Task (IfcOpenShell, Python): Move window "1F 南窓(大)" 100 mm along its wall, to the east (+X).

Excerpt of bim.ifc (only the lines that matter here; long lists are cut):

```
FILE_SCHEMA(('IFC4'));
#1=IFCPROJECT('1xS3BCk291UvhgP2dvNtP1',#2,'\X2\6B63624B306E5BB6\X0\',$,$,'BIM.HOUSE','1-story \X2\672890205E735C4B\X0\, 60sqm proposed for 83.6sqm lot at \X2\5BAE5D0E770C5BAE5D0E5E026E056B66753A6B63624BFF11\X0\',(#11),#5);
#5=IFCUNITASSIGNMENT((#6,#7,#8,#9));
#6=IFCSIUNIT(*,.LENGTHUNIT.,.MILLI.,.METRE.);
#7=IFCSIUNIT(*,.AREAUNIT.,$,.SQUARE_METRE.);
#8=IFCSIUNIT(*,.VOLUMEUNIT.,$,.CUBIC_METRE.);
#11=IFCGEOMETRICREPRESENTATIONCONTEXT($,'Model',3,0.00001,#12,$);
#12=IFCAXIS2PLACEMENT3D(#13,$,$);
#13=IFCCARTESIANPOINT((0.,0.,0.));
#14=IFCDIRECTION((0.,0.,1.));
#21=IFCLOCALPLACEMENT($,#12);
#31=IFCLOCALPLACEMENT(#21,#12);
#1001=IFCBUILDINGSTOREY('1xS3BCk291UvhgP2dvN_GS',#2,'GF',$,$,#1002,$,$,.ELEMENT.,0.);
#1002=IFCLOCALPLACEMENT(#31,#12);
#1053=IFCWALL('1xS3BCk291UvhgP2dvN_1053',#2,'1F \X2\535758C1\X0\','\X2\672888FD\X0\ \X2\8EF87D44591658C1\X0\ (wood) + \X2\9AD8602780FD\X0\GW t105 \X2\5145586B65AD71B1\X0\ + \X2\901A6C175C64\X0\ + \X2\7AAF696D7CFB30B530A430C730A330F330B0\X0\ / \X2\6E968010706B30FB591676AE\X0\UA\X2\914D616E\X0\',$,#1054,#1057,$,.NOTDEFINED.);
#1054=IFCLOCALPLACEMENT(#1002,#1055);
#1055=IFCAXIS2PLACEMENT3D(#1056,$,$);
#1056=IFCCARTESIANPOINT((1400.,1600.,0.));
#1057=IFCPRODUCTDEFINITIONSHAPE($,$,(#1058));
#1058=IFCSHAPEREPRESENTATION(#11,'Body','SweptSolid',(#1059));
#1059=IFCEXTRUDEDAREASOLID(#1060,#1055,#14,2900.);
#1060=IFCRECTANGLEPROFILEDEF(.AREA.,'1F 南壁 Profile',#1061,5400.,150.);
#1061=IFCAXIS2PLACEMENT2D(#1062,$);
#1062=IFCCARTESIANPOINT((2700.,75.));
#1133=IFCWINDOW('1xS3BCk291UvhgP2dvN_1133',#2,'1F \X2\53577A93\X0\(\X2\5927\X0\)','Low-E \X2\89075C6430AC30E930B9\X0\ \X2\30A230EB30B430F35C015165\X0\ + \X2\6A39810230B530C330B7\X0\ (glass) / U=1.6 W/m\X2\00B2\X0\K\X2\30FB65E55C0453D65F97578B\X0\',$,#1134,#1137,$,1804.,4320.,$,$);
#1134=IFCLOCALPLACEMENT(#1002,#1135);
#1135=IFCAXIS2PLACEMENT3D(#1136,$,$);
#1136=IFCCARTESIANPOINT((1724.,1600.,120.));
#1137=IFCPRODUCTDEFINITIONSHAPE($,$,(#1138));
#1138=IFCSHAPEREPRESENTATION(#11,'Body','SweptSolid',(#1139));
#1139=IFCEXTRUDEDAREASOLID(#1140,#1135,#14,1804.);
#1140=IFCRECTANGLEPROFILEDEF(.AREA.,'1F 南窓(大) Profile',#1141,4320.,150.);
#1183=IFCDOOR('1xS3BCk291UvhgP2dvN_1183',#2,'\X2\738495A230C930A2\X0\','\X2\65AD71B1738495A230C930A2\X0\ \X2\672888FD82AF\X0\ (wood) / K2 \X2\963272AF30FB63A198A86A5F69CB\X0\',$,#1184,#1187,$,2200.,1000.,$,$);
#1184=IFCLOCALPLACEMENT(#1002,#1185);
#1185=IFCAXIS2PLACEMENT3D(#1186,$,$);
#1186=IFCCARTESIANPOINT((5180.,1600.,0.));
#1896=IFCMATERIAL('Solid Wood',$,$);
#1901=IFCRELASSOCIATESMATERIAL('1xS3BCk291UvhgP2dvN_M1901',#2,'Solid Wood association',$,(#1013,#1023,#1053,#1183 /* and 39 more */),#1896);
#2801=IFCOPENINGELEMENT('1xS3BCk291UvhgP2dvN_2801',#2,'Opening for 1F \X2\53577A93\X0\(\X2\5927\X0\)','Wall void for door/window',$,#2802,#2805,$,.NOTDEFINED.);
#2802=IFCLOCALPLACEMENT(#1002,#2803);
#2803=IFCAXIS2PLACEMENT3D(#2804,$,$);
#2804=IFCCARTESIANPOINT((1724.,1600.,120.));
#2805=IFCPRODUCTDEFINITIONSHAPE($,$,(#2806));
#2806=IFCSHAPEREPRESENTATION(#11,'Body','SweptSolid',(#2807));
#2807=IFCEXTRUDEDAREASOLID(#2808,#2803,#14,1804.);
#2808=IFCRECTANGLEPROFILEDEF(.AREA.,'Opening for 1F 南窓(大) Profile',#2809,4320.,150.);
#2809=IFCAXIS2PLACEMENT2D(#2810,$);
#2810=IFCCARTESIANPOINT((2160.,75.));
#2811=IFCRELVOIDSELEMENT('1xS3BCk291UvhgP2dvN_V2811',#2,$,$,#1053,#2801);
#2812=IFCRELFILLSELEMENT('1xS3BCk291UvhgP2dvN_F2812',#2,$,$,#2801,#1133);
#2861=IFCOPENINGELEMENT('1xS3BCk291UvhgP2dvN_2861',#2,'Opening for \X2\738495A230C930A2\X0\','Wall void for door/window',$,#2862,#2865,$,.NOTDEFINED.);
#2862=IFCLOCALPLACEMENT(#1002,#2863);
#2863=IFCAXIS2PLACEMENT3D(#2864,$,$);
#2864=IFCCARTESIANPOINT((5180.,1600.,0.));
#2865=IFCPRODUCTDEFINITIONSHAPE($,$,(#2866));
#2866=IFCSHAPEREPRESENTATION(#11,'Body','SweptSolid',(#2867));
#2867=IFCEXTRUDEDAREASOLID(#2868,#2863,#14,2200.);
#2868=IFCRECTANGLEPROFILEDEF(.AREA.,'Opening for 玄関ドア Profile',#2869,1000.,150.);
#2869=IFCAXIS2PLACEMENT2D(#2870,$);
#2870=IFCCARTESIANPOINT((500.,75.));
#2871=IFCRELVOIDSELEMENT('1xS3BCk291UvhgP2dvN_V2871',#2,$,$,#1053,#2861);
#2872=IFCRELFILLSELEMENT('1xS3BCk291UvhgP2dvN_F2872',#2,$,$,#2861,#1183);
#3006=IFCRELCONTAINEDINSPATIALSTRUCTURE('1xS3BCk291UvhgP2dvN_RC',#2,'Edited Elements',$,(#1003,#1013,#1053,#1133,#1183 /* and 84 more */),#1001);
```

```python
import ifcopenshell
import ifcopenshell.api.geometry
import ifcopenshell.util.placement
import ifcopenshell.util.unit

model = ifcopenshell.open("bim.ifc")
unit_scale = ifcopenshell.util.unit.calculate_unit_scale(model)

window = model.by_guid("1xS3BCk291UvhgP2dvN_1133")
opening = window.FillsVoids[0].RelatingOpeningElement
wall = opening.VoidsElements[0].RelatingBuildingElement

wall_matrix = ifcopenshell.util.placement.get_local_placement(wall.ObjectPlacement)
shift = wall_matrix[:3, 0] * 0.1 / unit_scale
before = ifcopenshell.util.placement.get_local_placement(window.ObjectPlacement)[:3, 3].copy()

# The window is not placed relative to its opening, so move both.
for product in (opening, window):
    matrix = ifcopenshell.util.placement.get_local_placement(product.ObjectPlacement)
    matrix[:3, 3] += shift
    ifcopenshell.api.geometry.edit_object_placement(model, product=product, matrix=matrix, is_si=False)

after = ifcopenshell.util.placement.get_local_placement(window.ObjectPlacement)[:3, 3]
print("window moved by", (after - before).round(3) + 0.0)

model.write("bim_edited.ifc")
```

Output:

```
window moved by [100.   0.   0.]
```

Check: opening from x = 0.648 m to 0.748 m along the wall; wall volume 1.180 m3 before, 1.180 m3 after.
